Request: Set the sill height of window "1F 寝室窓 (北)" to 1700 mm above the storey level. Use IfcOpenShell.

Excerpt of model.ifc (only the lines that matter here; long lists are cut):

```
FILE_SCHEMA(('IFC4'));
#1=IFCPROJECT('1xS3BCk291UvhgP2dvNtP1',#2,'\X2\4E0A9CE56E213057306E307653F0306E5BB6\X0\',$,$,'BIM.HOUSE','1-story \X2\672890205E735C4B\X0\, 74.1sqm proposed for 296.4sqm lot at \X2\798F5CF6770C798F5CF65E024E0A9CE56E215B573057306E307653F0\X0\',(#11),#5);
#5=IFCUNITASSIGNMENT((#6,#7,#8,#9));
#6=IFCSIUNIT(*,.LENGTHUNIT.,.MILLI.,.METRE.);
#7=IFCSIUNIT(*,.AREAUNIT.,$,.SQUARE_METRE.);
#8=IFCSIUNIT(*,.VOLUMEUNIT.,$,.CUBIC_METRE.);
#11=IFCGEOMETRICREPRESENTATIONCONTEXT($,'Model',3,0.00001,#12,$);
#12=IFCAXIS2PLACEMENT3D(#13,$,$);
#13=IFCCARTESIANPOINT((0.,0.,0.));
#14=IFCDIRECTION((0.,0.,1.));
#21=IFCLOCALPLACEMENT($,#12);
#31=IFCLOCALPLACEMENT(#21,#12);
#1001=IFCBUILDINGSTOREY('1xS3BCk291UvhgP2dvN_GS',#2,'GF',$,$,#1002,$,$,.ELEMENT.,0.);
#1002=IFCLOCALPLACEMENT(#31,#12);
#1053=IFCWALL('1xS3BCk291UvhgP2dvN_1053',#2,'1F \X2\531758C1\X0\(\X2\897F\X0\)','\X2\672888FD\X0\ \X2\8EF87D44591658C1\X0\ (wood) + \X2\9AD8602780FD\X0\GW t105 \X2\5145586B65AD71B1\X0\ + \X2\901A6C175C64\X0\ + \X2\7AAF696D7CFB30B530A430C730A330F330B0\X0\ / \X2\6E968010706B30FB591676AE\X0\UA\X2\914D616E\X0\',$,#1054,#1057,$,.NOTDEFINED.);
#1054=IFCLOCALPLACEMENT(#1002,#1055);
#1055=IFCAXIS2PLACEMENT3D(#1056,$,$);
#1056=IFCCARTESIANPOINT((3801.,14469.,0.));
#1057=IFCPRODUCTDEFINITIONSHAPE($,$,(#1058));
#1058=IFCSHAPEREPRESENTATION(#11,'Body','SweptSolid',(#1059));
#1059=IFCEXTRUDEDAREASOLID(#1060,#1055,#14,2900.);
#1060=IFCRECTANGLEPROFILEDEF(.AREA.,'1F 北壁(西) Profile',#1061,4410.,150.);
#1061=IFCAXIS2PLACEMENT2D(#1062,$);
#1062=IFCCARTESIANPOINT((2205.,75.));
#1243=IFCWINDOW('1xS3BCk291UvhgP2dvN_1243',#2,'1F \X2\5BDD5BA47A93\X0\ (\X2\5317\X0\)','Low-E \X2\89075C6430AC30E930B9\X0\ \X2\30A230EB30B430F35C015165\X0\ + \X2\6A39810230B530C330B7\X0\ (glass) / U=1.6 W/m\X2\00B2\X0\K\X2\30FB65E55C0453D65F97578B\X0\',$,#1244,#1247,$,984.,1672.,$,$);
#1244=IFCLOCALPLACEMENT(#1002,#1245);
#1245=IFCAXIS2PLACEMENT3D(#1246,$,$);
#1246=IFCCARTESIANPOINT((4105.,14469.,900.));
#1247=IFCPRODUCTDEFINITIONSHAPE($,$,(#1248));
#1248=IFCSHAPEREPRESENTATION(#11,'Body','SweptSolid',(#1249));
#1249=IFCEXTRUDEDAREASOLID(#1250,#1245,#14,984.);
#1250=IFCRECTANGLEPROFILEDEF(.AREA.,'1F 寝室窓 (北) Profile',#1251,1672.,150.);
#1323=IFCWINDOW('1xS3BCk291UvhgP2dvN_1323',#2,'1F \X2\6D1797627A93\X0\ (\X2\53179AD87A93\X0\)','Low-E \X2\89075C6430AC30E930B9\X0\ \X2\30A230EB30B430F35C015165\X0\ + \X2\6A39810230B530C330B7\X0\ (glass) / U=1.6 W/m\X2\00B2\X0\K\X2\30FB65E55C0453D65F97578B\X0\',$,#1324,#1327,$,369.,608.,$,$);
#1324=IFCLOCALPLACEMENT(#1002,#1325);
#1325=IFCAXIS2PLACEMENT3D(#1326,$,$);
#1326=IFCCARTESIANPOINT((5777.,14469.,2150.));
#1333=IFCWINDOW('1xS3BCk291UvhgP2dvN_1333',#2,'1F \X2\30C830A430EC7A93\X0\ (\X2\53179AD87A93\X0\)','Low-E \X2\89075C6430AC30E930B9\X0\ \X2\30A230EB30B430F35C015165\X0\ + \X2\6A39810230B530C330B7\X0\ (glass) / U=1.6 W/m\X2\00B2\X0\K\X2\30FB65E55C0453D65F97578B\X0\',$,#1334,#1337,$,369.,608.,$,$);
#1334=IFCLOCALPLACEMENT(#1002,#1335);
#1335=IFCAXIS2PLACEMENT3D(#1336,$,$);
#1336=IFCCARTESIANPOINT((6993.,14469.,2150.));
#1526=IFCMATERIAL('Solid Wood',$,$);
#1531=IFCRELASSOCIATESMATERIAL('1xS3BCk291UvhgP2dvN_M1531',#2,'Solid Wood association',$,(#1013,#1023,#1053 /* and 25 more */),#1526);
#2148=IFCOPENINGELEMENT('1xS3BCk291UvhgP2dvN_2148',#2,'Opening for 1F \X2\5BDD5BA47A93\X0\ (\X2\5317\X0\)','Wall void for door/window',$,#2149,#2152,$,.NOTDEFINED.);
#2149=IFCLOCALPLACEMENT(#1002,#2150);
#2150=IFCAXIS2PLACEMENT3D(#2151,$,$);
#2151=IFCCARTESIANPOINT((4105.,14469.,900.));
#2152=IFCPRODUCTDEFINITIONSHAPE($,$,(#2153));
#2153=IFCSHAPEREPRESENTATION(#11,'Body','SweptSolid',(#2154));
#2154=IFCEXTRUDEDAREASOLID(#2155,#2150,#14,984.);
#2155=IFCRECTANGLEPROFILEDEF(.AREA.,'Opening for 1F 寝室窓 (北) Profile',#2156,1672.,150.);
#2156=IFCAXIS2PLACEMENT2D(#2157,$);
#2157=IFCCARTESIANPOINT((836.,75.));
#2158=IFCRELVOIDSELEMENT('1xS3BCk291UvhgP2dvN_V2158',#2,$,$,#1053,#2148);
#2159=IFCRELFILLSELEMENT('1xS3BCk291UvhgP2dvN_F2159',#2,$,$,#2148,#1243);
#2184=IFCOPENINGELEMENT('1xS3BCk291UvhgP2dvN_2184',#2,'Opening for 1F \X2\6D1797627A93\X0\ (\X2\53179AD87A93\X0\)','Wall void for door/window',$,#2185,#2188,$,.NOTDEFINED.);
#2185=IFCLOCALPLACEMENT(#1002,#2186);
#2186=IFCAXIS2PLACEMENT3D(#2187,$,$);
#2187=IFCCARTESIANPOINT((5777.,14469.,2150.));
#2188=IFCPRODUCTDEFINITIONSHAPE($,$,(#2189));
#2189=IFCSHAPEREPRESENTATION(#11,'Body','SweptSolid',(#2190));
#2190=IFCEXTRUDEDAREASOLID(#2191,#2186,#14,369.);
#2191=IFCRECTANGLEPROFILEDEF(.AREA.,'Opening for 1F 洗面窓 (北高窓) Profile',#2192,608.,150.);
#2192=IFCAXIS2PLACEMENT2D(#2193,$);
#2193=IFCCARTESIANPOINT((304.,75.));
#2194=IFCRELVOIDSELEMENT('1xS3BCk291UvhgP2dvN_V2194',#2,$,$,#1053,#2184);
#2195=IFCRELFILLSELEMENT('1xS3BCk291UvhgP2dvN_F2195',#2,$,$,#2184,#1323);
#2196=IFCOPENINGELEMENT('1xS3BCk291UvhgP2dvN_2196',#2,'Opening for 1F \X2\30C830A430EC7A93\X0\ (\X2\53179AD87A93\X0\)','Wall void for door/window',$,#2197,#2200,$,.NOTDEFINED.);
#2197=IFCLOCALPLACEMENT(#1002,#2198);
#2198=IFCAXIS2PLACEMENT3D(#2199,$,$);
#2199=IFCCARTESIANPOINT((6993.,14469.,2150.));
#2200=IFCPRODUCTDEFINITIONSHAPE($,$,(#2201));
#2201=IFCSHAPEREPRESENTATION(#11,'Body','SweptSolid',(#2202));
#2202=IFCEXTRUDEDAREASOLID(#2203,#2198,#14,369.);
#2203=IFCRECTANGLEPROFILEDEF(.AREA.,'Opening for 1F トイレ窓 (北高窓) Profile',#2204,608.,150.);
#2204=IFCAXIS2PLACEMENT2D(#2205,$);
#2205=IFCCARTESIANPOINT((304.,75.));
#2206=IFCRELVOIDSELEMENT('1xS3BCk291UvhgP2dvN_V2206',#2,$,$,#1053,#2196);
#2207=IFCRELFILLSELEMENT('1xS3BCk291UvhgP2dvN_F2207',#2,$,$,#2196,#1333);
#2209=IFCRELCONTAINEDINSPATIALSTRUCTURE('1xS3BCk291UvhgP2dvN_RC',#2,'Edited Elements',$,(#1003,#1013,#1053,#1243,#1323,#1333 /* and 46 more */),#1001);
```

```python
import numpy as np
import ifcopenshell
import ifcopenshell.api.geometry
import ifcopenshell.geom
import ifcopenshell.util.element
import ifcopenshell.util.placement
import ifcopenshell.util.shape
import ifcopenshell.util.unit

model = ifcopenshell.open("model.ifc")
unit_scale = ifcopenshell.util.unit.calculate_unit_scale(model)

window = model.by_guid("1xS3BCk291UvhgP2dvN_1243")
opening = window.FillsVoids[0].RelatingOpeningElement
storey = ifcopenshell.util.element.get_container(window, ifc_class="IfcBuildingStorey")
level = ifcopenshell.util.placement.get_local_placement(storey.ObjectPlacement)[2, 3]

# The opening's origin need not be at the sill, so measure its lowest point.
shape = ifcopenshell.geom.create_shape(ifcopenshell.geom.settings(), opening)
bottom = ifcopenshell.util.shape.get_shape_bottom_elevation(shape, shape.geometry) / unit_scale
dz = level + 1.7 / unit_scale - bottom

shift = np.array([0.0, 0.0, dz])
# The window is not placed relative to its opening, so move both.
for product in (opening, window):
    matrix = ifcopenshell.util.placement.get_local_placement(product.ObjectPlacement)
    matrix[:3, 3] += shift
    ifcopenshell.api.geometry.edit_object_placement(model, product=product, matrix=matrix, is_si=False)

print(f"moved by {dz * unit_scale:+.3f} m")

model.write("model-out.ifc")
```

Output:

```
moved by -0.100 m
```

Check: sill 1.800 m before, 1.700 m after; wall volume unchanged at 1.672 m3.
